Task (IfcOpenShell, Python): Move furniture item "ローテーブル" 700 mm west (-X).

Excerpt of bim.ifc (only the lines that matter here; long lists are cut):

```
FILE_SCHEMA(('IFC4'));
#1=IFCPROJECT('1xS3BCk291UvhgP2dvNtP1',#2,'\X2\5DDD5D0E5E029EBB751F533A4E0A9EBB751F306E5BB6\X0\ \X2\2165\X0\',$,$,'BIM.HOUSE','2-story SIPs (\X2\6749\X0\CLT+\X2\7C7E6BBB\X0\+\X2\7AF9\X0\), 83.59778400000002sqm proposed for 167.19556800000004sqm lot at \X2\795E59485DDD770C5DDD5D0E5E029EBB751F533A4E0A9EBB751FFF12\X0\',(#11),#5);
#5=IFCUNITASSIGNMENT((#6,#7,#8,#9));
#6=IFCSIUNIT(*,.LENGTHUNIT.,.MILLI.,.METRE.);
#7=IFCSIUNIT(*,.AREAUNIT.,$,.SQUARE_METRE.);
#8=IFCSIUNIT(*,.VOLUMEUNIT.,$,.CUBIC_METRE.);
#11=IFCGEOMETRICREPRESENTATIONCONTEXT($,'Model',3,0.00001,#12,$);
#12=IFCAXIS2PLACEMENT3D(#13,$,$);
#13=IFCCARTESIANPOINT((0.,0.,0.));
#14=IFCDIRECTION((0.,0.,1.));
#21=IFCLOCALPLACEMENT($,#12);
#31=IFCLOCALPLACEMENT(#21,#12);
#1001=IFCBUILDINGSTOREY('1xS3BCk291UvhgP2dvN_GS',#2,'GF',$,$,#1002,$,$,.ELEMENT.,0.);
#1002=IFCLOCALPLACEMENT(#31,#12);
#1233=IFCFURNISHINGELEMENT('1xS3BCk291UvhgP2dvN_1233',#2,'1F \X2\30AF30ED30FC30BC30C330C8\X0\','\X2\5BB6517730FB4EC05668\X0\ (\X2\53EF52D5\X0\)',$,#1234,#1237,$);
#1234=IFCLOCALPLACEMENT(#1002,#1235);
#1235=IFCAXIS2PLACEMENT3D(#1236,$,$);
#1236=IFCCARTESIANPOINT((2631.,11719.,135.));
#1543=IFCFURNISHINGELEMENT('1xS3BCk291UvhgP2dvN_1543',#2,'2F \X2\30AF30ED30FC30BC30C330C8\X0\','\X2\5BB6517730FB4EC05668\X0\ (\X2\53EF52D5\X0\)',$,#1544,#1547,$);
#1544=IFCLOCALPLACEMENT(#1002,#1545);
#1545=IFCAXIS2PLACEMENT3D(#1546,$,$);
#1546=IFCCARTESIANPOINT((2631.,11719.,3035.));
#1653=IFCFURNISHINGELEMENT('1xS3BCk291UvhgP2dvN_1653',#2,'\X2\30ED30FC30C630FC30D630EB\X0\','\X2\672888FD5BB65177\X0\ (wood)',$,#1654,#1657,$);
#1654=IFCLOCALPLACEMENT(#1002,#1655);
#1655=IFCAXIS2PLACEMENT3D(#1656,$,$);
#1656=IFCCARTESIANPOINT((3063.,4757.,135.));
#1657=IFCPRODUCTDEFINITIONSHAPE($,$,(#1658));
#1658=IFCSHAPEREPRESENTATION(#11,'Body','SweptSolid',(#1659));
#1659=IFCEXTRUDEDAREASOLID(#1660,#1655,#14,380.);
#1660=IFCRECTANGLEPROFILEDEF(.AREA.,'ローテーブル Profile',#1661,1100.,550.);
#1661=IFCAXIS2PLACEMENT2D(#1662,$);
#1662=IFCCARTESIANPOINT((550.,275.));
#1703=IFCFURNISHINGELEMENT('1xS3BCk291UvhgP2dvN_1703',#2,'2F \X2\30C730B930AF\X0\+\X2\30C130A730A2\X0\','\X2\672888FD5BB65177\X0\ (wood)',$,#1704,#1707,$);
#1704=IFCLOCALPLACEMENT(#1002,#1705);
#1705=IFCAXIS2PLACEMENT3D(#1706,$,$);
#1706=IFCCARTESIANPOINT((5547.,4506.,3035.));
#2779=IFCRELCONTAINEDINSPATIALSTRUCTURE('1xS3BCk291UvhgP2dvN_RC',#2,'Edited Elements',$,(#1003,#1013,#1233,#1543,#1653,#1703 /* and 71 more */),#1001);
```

```python
import ifcopenshell
import ifcopenshell.api.geometry
import ifcopenshell.util.placement
import ifcopenshell.util.unit

model = ifcopenshell.open("bim.ifc")
unit_scale = ifcopenshell.util.unit.calculate_unit_scale(model)

item = model.by_id(1653)
matrix = ifcopenshell.util.placement.get_local_placement(item.ObjectPlacement)
matrix[0, 3] -= 0.7 / unit_scale
ifcopenshell.api.geometry.edit_object_placement(model, product=item, matrix=matrix, is_si=False)

print(ifcopenshell.util.placement.get_local_placement(item.ObjectPlacement).round(3) + 0.0)

model.write("bim_updated.ifc")
```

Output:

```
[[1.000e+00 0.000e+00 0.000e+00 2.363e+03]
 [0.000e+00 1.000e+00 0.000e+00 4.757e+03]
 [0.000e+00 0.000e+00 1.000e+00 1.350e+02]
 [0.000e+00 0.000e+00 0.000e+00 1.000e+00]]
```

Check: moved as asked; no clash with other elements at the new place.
